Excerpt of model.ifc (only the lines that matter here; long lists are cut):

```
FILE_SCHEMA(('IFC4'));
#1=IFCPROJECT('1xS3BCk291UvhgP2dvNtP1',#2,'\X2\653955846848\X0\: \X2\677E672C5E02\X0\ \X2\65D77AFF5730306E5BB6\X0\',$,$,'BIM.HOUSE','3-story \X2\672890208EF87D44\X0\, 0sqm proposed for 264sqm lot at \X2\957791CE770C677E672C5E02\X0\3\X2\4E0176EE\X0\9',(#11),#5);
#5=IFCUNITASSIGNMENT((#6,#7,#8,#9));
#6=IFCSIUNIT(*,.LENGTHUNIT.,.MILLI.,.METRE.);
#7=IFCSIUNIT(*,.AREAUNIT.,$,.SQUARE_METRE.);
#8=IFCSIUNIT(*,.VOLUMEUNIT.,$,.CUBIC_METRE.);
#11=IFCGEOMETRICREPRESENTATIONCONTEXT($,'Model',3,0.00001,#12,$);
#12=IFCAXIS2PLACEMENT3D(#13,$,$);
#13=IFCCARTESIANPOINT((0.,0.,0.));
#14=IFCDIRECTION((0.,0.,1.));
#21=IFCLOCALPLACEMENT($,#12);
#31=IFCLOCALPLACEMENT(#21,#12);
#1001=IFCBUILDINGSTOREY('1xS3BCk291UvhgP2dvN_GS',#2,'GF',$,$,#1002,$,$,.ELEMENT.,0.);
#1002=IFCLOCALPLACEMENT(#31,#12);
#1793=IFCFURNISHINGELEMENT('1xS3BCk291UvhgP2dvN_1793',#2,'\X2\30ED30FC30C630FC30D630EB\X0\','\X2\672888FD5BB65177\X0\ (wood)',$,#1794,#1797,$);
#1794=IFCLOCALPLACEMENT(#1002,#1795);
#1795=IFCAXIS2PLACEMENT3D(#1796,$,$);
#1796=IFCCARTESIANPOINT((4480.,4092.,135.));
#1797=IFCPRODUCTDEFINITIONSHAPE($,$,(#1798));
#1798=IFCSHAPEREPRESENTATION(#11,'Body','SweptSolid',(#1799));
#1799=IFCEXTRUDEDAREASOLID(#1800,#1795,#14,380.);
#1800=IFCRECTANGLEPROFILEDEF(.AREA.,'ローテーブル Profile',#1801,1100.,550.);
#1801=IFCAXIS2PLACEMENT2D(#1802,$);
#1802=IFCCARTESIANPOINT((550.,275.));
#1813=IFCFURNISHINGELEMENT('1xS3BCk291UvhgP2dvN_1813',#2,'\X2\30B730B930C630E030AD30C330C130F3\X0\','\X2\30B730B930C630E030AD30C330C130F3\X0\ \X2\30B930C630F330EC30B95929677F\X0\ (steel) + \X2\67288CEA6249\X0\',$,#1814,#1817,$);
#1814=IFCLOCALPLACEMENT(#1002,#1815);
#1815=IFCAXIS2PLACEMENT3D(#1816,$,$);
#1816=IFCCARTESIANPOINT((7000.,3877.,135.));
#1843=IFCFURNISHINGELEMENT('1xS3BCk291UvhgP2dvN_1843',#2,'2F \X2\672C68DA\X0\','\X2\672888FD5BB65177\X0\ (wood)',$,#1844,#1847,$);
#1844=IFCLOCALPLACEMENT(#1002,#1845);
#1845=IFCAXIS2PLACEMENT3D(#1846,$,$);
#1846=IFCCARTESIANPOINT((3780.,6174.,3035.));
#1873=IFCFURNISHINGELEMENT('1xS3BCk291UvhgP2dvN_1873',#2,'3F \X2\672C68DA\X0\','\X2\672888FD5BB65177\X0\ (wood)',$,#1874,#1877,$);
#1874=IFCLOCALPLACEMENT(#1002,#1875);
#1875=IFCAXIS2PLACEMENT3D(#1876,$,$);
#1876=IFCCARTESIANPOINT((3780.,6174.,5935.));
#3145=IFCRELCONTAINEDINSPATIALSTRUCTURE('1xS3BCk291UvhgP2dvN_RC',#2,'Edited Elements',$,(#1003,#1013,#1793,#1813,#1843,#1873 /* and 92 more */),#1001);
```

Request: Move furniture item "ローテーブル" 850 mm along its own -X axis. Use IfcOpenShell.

```python
import ifcopenshell
import ifcopenshell.api.geometry
import ifcopenshell.util.placement

model = ifcopenshell.open("model.ifc")

item = model.by_guid("1xS3BCk291UvhgP2dvN_1793")
matrix = ifcopenshell.util.placement.get_local_placement(item.ObjectPlacement)
matrix[:3, 3] -= matrix[:3, 0] * 850.0
ifcopenshell.api.geometry.edit_object_placement(model, product=item, matrix=matrix, is_si=False)

print(ifcopenshell.util.placement.get_local_placement(item.ObjectPlacement).round(3) + 0.0)

model.write("model-out.ifc")
```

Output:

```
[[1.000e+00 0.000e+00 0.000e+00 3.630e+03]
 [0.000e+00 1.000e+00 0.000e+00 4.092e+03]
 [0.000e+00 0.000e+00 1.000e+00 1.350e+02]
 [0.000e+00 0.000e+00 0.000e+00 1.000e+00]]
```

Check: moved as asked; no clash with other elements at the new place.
